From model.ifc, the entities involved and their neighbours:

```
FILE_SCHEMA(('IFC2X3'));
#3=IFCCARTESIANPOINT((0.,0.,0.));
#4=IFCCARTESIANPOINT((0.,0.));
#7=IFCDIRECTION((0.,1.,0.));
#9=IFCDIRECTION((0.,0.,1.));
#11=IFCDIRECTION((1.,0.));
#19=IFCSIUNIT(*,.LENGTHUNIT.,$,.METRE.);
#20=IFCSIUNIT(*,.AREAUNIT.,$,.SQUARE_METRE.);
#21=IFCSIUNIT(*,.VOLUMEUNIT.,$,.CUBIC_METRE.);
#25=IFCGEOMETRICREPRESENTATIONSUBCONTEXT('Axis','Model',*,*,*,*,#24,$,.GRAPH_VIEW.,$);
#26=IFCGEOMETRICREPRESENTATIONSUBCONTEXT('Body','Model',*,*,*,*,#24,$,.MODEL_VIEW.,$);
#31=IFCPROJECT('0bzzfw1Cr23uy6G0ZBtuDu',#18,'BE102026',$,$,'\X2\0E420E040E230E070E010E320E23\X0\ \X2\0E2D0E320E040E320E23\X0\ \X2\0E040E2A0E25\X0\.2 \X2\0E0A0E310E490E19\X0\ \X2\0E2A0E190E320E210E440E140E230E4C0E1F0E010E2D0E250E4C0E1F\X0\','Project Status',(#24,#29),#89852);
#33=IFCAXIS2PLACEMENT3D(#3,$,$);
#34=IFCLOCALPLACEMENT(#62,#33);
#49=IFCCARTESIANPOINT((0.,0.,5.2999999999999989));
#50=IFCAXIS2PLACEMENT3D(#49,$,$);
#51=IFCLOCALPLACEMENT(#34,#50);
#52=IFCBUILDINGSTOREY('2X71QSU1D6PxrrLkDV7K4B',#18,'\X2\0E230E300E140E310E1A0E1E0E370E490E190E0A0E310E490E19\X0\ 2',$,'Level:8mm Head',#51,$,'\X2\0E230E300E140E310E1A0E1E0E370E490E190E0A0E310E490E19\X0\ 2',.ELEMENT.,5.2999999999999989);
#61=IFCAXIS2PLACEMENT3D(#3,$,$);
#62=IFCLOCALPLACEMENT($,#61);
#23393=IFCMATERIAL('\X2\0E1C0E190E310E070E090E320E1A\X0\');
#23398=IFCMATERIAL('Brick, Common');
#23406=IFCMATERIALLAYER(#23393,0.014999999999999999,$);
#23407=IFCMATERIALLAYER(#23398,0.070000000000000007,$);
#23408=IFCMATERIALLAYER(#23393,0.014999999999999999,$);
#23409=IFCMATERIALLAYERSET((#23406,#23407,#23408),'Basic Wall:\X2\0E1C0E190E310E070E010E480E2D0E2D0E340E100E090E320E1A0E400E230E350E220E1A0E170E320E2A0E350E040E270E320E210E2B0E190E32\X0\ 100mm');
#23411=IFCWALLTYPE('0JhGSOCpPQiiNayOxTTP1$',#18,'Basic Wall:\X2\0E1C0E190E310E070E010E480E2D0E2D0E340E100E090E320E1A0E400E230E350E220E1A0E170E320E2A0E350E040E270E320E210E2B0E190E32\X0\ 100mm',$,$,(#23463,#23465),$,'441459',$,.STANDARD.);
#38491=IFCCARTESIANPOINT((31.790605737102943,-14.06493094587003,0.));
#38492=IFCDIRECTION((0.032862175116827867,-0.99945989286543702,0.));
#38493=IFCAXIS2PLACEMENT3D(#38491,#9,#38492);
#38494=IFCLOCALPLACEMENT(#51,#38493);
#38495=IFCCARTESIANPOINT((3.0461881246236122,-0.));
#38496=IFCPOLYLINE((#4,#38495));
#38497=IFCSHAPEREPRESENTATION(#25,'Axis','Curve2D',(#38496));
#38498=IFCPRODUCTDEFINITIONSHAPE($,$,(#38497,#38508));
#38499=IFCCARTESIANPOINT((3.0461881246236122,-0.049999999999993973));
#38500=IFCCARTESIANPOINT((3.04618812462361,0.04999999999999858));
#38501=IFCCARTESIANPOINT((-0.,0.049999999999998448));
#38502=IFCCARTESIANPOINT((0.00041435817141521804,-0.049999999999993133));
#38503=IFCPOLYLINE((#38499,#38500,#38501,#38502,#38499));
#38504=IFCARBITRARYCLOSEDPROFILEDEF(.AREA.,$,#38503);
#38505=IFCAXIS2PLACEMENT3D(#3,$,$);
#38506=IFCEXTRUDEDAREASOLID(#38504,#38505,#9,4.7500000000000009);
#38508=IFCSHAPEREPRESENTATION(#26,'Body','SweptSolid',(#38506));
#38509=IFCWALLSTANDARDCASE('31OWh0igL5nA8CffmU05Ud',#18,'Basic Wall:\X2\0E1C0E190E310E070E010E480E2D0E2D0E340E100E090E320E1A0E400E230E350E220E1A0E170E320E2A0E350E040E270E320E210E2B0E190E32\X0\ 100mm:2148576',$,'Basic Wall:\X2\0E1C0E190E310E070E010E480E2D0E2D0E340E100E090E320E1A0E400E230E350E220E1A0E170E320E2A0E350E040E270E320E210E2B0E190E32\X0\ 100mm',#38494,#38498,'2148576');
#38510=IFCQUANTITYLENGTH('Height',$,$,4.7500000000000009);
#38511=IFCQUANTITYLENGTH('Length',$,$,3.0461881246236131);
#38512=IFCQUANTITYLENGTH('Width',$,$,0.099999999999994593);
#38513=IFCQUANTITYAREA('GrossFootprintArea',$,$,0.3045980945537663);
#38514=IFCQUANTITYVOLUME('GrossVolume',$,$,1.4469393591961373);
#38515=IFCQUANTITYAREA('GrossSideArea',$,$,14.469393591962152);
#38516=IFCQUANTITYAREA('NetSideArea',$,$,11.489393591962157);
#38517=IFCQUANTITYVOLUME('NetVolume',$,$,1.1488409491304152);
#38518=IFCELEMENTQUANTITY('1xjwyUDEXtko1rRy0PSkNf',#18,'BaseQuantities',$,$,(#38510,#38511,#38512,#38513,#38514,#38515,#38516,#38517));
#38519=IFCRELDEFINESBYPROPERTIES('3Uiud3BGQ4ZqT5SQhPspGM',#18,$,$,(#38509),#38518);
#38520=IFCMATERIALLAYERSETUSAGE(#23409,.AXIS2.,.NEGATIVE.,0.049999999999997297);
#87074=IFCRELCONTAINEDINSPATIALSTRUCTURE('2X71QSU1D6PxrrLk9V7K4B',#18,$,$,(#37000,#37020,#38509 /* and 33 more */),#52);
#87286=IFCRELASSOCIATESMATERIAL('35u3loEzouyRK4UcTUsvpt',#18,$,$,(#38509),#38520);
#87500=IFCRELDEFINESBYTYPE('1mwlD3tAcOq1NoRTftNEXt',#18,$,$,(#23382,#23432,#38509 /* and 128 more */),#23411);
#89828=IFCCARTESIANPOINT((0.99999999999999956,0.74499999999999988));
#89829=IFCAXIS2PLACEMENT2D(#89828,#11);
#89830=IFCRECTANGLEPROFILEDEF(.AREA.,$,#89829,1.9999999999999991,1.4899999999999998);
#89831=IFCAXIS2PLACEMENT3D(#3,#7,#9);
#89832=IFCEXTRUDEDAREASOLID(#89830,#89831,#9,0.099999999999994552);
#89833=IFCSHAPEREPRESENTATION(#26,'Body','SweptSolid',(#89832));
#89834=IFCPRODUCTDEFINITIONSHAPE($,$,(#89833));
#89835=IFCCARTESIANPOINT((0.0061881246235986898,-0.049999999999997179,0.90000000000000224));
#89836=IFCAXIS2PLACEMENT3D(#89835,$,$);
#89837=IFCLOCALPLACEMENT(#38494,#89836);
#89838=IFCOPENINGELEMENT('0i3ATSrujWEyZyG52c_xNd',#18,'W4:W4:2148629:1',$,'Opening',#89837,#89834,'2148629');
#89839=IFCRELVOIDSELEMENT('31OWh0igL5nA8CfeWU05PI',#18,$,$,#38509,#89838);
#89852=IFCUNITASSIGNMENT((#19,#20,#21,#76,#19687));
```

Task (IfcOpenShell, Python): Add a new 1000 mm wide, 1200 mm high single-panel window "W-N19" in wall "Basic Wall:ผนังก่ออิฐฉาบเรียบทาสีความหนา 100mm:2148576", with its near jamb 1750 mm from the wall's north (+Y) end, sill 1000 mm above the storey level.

```python
import numpy as np
import ifcopenshell
import ifcopenshell.api.feature
import ifcopenshell.api.geometry
import ifcopenshell.api.pset
import ifcopenshell.api.root
import ifcopenshell.api.spatial
import ifcopenshell.api.type
import ifcopenshell.geom
import ifcopenshell.util.element
import ifcopenshell.util.placement
import ifcopenshell.util.representation
import ifcopenshell.util.shape
import ifcopenshell.util.unit

model = ifcopenshell.open("model.ifc")
unit_scale = ifcopenshell.util.unit.calculate_unit_scale(model)
area_scale = ifcopenshell.util.unit.calculate_unit_scale(model, "AREAUNIT")
volume_scale = ifcopenshell.util.unit.calculate_unit_scale(model, "VOLUMEUNIT")
settings = ifcopenshell.geom.settings()


def volume(element):
    """Net volume in cubic metres, openings subtracted."""
    shape = ifcopenshell.geom.create_shape(settings, element)
    return ifcopenshell.util.shape.get_volume(shape.geometry)


wall = model.by_id(38509)
storey = ifcopenshell.util.element.get_container(wall, ifc_class="IfcBuildingStorey")
context = ifcopenshell.util.representation.get_context(model, "Model", "Body", "MODEL_VIEW")
before = volume(wall)

width, height, from_end, sill = 1, 1.2, 1.75, 1  # metres

# The wall runs along its own X axis, and the end named is its -X end.
wall_shape = ifcopenshell.geom.create_shape(settings, wall)
x, y, z = ifcopenshell.util.shape.get_vertices(wall_shape.geometry).T
start = x.min() + from_end
face, thickness = float(y.min()), float(y.max() - y.min())
wall_matrix = ifcopenshell.util.placement.get_local_placement(wall.ObjectPlacement)
level = ifcopenshell.util.placement.get_local_placement(storey.ObjectPlacement)[2, 3]


def in_wall(x, y):
    """Placement at x, y metres in the wall's axes, at sill height."""
    matrix = wall_matrix.copy()
    matrix[:, 3] = wall_matrix @ np.array([x / unit_scale, y / unit_scale, 0.0, 1.0])
    matrix[2, 3] = level + sill / unit_scale
    return matrix


# Opening: a box that overshoots both wall faces by 50 mm.
opening = ifcopenshell.api.root.create_entity(model, ifc_class="IfcOpeningElement")
box = ifcopenshell.api.geometry.add_wall_representation(
    model, context=context, length=width, height=height, thickness=thickness + 0.1
)
ifcopenshell.api.geometry.assign_representation(model, product=opening, representation=box)
ifcopenshell.api.geometry.edit_object_placement(model, product=opening, matrix=in_wall(start, face - 0.05), is_si=False)
ifcopenshell.api.feature.add_feature(model, feature=opening, element=wall)

window = ifcopenshell.api.root.create_entity(model, ifc_class="IfcWindow", name="W-N19")
window.OverallWidth, window.OverallHeight = width / unit_scale, height / unit_scale
body = ifcopenshell.api.geometry.add_window_representation(
    model,
    context=context,
    overall_width=window.OverallWidth,
    overall_height=window.OverallHeight,
    partition_type="SINGLE_PANEL",
)
ifcopenshell.api.geometry.assign_representation(model, product=window, representation=body)
ifcopenshell.api.spatial.assign_container(model, products=[window], relating_structure=storey)
fills = ifcopenshell.api.feature.add_filling(model, opening=opening, element=window)
fills.OwnerHistory = window.OwnerHistory  # required in IFC2X3

# IFC2X3 keeps the operation on the window style.
style = ifcopenshell.api.root.create_entity(model, ifc_class="IfcWindowStyle", name="W-N19")
style.OperationType, style.ConstructionType = "SINGLE_PANEL", "NOTDEFINED"
style.ParameterTakesPrecedence = style.Sizeable = False
ifcopenshell.api.type.assign_type(model, related_objects=[window], relating_type=style)

# Centre the window in the wall's thickness.
ifcopenshell.api.geometry.edit_object_placement(model, product=window, matrix=in_wall(start, face), is_si=False)
window_shape = ifcopenshell.geom.create_shape(settings, window)
depth = ifcopenshell.util.shape.get_vertices(window_shape.geometry)[:, 1]
offset = face + thickness / 2 - (depth.min() + depth.max()) / 2
ifcopenshell.api.geometry.edit_object_placement(model, product=window, matrix=in_wall(start, offset), is_si=False)

after = volume(wall)

# Update the wall's stored quantities.
qto = model.by_id(ifcopenshell.util.element.get_pset(wall, "BaseQuantities", should_inherit=False)["id"])
ifcopenshell.api.pset.edit_qto(model, qto=qto, properties={
    "NetSideArea": after / thickness / area_scale,
    "NetVolume": after / volume_scale,
})

print(f"wall volume {before:.3f} -> {after:.3f} m3")

model.write("model_updated.ifc")
```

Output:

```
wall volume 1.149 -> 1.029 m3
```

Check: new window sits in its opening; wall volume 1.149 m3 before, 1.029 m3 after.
